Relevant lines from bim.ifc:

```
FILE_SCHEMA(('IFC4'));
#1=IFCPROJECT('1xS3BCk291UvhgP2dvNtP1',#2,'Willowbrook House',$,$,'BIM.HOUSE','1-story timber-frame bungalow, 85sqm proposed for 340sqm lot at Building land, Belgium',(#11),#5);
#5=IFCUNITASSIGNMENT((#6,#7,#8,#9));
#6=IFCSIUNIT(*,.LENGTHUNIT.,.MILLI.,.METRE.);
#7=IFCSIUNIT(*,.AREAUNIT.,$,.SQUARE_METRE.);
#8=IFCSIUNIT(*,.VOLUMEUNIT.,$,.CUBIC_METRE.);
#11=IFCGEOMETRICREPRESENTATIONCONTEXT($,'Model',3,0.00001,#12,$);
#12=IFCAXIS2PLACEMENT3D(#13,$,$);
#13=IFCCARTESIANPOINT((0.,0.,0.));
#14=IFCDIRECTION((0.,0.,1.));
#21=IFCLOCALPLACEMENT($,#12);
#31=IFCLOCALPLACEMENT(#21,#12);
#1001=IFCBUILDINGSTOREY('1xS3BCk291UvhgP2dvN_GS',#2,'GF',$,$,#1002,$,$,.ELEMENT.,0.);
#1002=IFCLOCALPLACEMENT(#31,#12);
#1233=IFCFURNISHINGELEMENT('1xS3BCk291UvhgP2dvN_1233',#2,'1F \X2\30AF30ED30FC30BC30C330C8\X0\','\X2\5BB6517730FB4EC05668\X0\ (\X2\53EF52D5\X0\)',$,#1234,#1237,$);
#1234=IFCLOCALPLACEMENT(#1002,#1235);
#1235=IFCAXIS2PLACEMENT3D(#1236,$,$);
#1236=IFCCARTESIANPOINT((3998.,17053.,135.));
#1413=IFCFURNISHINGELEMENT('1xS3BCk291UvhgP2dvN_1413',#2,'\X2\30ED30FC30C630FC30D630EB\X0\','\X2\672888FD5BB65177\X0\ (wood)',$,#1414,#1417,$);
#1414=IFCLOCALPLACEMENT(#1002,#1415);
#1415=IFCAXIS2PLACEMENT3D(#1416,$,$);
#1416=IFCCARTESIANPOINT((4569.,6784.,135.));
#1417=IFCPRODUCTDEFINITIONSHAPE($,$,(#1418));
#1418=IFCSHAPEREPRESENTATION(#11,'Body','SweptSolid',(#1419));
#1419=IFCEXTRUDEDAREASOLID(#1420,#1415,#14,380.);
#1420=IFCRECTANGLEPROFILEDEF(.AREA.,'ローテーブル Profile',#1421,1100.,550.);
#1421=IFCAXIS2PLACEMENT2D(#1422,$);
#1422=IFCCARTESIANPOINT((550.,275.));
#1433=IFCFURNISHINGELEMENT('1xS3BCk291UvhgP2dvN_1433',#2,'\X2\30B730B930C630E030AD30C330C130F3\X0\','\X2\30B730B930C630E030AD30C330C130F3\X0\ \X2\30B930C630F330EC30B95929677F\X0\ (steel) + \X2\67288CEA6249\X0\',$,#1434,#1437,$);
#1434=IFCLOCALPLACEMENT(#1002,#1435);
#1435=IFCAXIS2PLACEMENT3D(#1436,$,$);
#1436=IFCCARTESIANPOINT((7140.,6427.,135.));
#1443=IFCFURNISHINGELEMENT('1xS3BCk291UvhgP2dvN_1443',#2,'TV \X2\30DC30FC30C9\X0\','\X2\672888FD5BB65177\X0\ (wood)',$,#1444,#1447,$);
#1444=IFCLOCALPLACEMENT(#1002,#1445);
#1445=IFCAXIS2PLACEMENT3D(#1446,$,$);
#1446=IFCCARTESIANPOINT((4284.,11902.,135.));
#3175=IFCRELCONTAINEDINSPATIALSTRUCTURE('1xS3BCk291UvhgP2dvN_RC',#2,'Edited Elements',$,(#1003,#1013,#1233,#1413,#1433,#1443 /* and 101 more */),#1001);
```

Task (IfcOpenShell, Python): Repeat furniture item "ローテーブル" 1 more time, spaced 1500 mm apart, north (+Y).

```python
import numpy as np
import ifcopenshell
import ifcopenshell.api.geometry
import ifcopenshell.api.root
import ifcopenshell.util.element
import ifcopenshell.util.placement
import ifcopenshell.util.unit

model = ifcopenshell.open("bim.ifc")
unit_scale = ifcopenshell.util.unit.calculate_unit_scale(model)


def reuse_history(source, copy):
    """copy_class also copies each property set's owner history, people and application; keep the originals."""
    for rel in copy.IsDefinedBy:
        if rel.is_a("IfcRelDefinesByProperties") and (history := rel.RelatingPropertyDefinition.OwnerHistory):
            rel.RelatingPropertyDefinition.OwnerHistory = source.OwnerHistory
            ifcopenshell.util.element.remove_deep2(model, history)


source = model.by_guid("1xS3BCk291UvhgP2dvN_1413")
base = ifcopenshell.util.placement.get_local_placement(source.ObjectPlacement)
step = np.array([0.0, 1.0, 0.0]) * 1.5 / unit_scale

for i in range(1, 2):
    copy = ifcopenshell.api.root.copy_class(model, product=source)
    copy.Representation = ifcopenshell.util.element.copy_deep(
        model, source.Representation, exclude=["IfcGeometricRepresentationContext", "IfcRepresentationMap"]
    )
    reuse_history(source, copy)
    matrix = base.copy()
    matrix[:3, 3] += i * step
    print("added at", matrix[:3, 3].round(3) + 0.0)
    ifcopenshell.api.geometry.edit_object_placement(model, product=copy, matrix=matrix, is_si=False)

model.write("bim_edited.ifc")
```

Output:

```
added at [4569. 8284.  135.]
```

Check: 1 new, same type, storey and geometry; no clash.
